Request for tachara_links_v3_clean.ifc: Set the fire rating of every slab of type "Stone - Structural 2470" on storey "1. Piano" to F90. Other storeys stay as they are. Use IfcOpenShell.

First a look at what the model holds.

```python
import ifcopenshell
import ifcopenshell.util.element

model = ifcopenshell.open("tachara_links_v3_clean.ifc")
print(model.schema)
storey = next(s for s in model.by_type("IfcBuildingStorey") if s.Name == "1. Piano")
slabs = [e for e in ifcopenshell.util.element.get_decomposition(storey) if e.is_a("IfcSlab")]
seen = {}
for e in slabs:
    element_type = ifcopenshell.util.element.get_type(e)
    key = (element_type.Name if element_type != e and element_type else None, ifcopenshell.util.element.get_pset(e, "Pset_SlabCommon", "FireRating"))
    seen[key] = seen.get(key, 0) + 1
for (name, value), count in sorted(seen.items(), key=str):
    print(count, "x", name, "|", value)
```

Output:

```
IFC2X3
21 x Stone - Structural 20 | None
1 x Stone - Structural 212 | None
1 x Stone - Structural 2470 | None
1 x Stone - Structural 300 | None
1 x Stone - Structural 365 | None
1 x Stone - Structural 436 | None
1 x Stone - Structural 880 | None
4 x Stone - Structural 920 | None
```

```python
import ifcopenshell
import ifcopenshell.api.pset
import ifcopenshell.util.element

model = ifcopenshell.open("tachara_links_v3_clean.ifc")

storey = next(s for s in model.by_type("IfcBuildingStorey") if s.Name == "1. Piano")
slabs = [e for e in ifcopenshell.util.element.get_decomposition(storey) if e.is_a("IfcSlab")]

count = 0
for e in slabs:
    element_type = ifcopenshell.util.element.get_type(e)
    if element_type in (None, e) or element_type.Name != "Stone - Structural 2470":
        continue
    # add_pset returns the element's existing set when there is one.
    pset = ifcopenshell.api.pset.add_pset(model, product=e, name="Pset_SlabCommon")
    ifcopenshell.api.pset.edit_pset(model, pset=pset, properties={"FireRating": "F90"})
    count += 1

print(count, "slabs updated")

model.write("tachara_links_v3_clean_rev.ifc")
```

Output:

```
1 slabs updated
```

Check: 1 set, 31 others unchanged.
